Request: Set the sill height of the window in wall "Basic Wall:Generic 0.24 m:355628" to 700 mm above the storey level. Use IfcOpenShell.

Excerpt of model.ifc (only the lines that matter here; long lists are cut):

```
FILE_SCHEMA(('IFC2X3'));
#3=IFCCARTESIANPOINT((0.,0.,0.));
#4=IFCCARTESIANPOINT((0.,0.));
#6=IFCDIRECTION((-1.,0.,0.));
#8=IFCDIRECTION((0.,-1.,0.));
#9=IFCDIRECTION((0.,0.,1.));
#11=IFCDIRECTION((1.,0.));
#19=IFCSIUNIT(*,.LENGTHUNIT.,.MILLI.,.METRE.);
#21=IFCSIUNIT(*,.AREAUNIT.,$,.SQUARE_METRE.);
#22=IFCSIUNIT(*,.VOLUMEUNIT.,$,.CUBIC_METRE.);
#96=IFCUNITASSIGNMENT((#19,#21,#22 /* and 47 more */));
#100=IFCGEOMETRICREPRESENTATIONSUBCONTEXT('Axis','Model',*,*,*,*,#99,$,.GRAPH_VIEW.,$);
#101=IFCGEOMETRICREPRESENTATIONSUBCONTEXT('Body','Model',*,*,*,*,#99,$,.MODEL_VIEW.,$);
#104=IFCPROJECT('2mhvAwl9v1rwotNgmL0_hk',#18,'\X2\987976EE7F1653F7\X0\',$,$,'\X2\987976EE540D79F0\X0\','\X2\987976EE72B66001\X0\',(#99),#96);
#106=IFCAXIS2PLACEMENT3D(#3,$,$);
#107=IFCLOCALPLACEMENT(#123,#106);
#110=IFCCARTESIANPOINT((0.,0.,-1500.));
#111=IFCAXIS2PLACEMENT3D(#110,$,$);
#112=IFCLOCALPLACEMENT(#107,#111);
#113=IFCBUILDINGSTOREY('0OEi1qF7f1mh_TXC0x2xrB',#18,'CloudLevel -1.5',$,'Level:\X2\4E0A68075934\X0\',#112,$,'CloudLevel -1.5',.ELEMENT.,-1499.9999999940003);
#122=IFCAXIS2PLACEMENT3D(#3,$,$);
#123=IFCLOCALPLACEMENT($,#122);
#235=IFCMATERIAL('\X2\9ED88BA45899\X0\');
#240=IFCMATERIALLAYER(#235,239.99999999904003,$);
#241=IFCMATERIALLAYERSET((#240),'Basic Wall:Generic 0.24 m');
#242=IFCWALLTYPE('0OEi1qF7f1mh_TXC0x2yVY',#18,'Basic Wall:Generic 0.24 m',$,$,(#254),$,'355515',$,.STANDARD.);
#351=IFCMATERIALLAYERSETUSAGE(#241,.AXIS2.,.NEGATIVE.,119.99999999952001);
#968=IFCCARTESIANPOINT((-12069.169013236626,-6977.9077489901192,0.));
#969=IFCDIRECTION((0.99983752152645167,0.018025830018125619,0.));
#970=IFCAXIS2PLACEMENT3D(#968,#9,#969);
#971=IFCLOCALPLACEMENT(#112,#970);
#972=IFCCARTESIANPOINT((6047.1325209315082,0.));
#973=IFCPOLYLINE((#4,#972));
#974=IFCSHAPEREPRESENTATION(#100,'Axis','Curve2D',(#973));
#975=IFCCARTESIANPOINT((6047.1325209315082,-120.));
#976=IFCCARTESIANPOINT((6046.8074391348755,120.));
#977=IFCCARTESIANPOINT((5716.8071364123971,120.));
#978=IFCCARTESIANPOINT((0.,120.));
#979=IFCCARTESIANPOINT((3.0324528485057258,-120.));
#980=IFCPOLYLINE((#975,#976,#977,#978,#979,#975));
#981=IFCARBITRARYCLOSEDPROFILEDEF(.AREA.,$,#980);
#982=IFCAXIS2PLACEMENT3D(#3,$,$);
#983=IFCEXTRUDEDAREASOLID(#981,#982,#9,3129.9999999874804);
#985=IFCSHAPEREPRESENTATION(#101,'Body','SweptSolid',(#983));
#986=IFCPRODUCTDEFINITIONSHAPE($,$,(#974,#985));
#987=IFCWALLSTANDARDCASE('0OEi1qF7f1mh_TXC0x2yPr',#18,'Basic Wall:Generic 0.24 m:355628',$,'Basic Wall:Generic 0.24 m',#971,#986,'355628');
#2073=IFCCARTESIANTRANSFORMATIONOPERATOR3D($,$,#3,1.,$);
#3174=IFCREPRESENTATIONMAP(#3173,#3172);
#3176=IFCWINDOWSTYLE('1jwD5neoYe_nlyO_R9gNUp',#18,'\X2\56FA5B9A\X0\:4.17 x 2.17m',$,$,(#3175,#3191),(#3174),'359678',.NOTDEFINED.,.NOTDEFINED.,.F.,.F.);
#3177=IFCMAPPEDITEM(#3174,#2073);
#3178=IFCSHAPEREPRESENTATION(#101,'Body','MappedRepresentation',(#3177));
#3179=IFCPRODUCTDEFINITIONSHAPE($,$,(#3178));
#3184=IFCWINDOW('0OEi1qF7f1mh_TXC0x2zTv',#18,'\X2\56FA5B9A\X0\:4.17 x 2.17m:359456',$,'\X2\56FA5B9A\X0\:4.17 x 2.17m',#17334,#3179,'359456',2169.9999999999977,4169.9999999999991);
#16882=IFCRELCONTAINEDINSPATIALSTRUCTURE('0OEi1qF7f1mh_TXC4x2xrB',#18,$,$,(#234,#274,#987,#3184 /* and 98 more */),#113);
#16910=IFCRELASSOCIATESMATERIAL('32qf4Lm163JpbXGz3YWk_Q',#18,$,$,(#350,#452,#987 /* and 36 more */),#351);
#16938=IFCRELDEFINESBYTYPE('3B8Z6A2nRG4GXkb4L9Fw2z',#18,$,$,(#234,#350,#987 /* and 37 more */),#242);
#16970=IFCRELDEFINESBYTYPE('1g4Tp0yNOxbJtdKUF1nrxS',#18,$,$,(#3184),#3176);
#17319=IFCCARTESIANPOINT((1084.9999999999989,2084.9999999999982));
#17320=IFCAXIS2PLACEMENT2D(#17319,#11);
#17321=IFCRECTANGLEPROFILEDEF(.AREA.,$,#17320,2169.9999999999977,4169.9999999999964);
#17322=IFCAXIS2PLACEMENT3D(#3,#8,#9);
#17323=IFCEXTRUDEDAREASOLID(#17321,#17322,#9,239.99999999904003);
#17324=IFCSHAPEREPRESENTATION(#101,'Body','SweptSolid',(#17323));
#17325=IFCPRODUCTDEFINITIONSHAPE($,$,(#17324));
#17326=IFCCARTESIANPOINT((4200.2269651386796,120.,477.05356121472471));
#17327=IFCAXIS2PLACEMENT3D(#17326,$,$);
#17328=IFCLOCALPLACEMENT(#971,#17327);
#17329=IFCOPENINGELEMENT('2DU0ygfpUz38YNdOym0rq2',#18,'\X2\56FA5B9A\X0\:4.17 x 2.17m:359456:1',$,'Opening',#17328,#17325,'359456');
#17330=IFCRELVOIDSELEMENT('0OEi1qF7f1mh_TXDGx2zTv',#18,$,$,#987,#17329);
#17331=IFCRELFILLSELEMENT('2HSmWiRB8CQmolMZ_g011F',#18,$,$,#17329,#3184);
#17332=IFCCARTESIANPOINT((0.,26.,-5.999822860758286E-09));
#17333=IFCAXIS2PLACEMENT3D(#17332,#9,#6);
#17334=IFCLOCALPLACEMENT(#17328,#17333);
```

```python
import numpy as np
import ifcopenshell
import ifcopenshell.api.geometry
import ifcopenshell.geom
import ifcopenshell.util.element
import ifcopenshell.util.placement
import ifcopenshell.util.shape
import ifcopenshell.util.unit

model = ifcopenshell.open("model.ifc")
unit_scale = ifcopenshell.util.unit.calculate_unit_scale(model)

window = model.by_guid("0OEi1qF7f1mh_TXC0x2zTv")
opening = window.FillsVoids[0].RelatingOpeningElement
storey = ifcopenshell.util.element.get_container(window, ifc_class="IfcBuildingStorey")
level = ifcopenshell.util.placement.get_local_placement(storey.ObjectPlacement)[2, 3]

# The opening's origin need not be at the sill, so measure its lowest point.
shape = ifcopenshell.geom.create_shape(ifcopenshell.geom.settings(), opening)
bottom = ifcopenshell.util.shape.get_shape_bottom_elevation(shape, shape.geometry) / unit_scale
dz = level + 700.0 - bottom

shift = np.array([0.0, 0.0, dz])
# The window is placed relative to its opening, so it follows when the opening moves.
matrix = ifcopenshell.util.placement.get_local_placement(opening.ObjectPlacement)
matrix[:3, 3] += shift
ifcopenshell.api.geometry.edit_object_placement(
    model, product=opening, matrix=matrix, is_si=False, should_transform_children=True
)

print(f"moved by {dz * unit_scale:+.3f} m")

model.write("model_updated.ifc")
```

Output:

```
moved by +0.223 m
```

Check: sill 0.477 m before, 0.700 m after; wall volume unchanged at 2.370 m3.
